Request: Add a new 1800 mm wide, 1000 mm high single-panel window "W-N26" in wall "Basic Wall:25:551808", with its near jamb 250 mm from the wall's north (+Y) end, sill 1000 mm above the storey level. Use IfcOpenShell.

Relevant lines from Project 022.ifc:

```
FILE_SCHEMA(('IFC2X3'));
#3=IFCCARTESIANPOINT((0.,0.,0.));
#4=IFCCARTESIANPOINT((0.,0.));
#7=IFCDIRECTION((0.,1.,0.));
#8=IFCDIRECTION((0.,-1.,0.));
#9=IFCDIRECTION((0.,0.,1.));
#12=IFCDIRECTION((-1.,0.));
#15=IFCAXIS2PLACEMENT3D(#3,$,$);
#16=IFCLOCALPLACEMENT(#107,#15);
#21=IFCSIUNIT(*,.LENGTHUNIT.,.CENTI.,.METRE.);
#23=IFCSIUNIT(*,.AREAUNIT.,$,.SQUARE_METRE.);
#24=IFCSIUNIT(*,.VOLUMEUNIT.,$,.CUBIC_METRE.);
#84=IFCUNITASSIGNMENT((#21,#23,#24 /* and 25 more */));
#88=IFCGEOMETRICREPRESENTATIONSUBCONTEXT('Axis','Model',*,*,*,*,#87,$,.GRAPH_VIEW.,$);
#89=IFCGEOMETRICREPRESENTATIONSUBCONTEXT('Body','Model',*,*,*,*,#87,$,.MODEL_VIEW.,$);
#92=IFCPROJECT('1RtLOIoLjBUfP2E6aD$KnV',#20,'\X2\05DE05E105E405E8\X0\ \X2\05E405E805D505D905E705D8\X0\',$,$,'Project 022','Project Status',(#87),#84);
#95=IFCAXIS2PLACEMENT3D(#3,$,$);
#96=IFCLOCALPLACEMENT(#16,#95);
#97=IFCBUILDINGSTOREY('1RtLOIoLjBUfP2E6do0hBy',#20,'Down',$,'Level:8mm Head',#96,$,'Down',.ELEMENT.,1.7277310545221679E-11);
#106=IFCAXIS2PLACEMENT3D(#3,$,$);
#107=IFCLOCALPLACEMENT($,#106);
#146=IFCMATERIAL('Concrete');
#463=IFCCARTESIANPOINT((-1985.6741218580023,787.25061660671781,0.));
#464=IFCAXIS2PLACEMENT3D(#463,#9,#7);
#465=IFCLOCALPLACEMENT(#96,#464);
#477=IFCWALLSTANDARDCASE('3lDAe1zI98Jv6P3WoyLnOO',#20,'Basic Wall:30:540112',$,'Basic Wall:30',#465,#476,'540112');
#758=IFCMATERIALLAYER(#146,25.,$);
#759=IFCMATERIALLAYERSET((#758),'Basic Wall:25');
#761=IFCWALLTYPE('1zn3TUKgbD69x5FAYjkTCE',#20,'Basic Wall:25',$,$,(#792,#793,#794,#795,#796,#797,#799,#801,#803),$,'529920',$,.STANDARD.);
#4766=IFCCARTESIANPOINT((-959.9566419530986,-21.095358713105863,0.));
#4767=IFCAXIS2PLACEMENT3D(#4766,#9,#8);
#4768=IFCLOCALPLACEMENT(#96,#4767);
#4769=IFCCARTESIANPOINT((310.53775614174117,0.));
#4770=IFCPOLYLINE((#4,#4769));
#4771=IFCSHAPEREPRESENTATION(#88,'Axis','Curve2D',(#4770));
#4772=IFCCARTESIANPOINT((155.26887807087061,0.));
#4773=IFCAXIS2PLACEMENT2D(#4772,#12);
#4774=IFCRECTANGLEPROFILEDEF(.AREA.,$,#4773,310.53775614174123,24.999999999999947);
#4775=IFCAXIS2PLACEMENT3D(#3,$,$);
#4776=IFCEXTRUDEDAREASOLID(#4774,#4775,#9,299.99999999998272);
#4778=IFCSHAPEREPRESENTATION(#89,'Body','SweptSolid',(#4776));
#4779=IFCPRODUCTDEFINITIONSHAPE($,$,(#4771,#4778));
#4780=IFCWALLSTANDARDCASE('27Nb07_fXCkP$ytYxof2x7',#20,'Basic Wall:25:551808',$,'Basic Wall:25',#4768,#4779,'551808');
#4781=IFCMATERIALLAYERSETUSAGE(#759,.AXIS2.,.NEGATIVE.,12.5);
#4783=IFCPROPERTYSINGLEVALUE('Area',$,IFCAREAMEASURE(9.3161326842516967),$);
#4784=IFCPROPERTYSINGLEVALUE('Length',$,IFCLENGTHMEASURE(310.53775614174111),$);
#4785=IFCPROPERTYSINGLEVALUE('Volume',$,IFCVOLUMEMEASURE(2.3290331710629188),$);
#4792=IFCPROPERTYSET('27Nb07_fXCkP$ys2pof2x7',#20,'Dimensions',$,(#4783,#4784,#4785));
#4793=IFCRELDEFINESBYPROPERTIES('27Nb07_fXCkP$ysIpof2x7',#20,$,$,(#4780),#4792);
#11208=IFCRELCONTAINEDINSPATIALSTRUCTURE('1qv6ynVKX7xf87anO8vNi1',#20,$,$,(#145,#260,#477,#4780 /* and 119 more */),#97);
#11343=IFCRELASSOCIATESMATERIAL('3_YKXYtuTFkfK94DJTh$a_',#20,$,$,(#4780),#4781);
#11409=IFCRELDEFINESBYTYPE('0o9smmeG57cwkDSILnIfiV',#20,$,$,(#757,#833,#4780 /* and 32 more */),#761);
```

```python
import numpy as np
import ifcopenshell
import ifcopenshell.api.feature
import ifcopenshell.api.geometry
import ifcopenshell.api.pset
import ifcopenshell.api.root
import ifcopenshell.api.spatial
import ifcopenshell.api.type
import ifcopenshell.geom
import ifcopenshell.util.element
import ifcopenshell.util.placement
import ifcopenshell.util.representation
import ifcopenshell.util.shape
import ifcopenshell.util.unit

model = ifcopenshell.open("Project 022.ifc")
unit_scale = ifcopenshell.util.unit.calculate_unit_scale(model)
area_scale = ifcopenshell.util.unit.calculate_unit_scale(model, "AREAUNIT")
volume_scale = ifcopenshell.util.unit.calculate_unit_scale(model, "VOLUMEUNIT")
settings = ifcopenshell.geom.settings()


def volume(element):
    """Net volume in cubic metres, openings subtracted."""
    shape = ifcopenshell.geom.create_shape(settings, element)
    return ifcopenshell.util.shape.get_volume(shape.geometry)


wall = model.by_guid("27Nb07_fXCkP$ytYxof2x7")
storey = ifcopenshell.util.element.get_container(wall, ifc_class="IfcBuildingStorey")
context = ifcopenshell.util.representation.get_context(model, "Model", "Body", "MODEL_VIEW")
before = volume(wall)

width, height, from_end, sill = 1.8, 1, 0.25, 1  # metres

# The wall runs along its own X axis, and the end named is its -X end.
wall_shape = ifcopenshell.geom.create_shape(settings, wall)
x, y, z = ifcopenshell.util.shape.get_vertices(wall_shape.geometry).T
start = x.min() + from_end
face, thickness = float(y.min()), float(y.max() - y.min())
wall_matrix = ifcopenshell.util.placement.get_local_placement(wall.ObjectPlacement)
level = ifcopenshell.util.placement.get_local_placement(storey.ObjectPlacement)[2, 3]


def in_wall(x, y):
    """Placement at x, y metres in the wall's axes, at sill height."""
    matrix = wall_matrix.copy()
    matrix[:, 3] = wall_matrix @ np.array([x / unit_scale, y / unit_scale, 0.0, 1.0])
    matrix[2, 3] = level + sill / unit_scale
    return matrix


# Opening: a box that overshoots both wall faces by 50 mm.
opening = ifcopenshell.api.root.create_entity(model, ifc_class="IfcOpeningElement")
box = ifcopenshell.api.geometry.add_wall_representation(
    model, context=context, length=width, height=height, thickness=thickness + 0.1
)
ifcopenshell.api.geometry.assign_representation(model, product=opening, representation=box)
ifcopenshell.api.geometry.edit_object_placement(model, product=opening, matrix=in_wall(start, face - 0.05), is_si=False)
ifcopenshell.api.feature.add_feature(model, feature=opening, element=wall)

window = ifcopenshell.api.root.create_entity(model, ifc_class="IfcWindow", name="W-N26")
window.OverallWidth, window.OverallHeight = width / unit_scale, height / unit_scale
body = ifcopenshell.api.geometry.add_window_representation(
    model,
    context=context,
    overall_width=window.OverallWidth,
    overall_height=window.OverallHeight,
    partition_type="SINGLE_PANEL",
)
ifcopenshell.api.geometry.assign_representation(model, product=window, representation=body)
ifcopenshell.api.spatial.assign_container(model, products=[window], relating_structure=storey)
fills = ifcopenshell.api.feature.add_filling(model, opening=opening, element=window)
fills.OwnerHistory = window.OwnerHistory  # required in IFC2X3

# IFC2X3 keeps the operation on the window style.
style = ifcopenshell.api.root.create_entity(model, ifc_class="IfcWindowStyle", name="W-N26")
style.OperationType, style.ConstructionType = "SINGLE_PANEL", "NOTDEFINED"
style.ParameterTakesPrecedence = style.Sizeable = False
ifcopenshell.api.type.assign_type(model, related_objects=[window], relating_type=style)

# Centre the window in the wall's thickness.
ifcopenshell.api.geometry.edit_object_placement(model, product=window, matrix=in_wall(start, face), is_si=False)
window_shape = ifcopenshell.geom.create_shape(settings, window)
depth = ifcopenshell.util.shape.get_vertices(window_shape.geometry)[:, 1]
offset = face + thickness / 2 - (depth.min() + depth.max()) / 2
ifcopenshell.api.geometry.edit_object_placement(model, product=window, matrix=in_wall(start, offset), is_si=False)

after = volume(wall)

# Update the wall's stored quantities.
pset = model.by_id(ifcopenshell.util.element.get_pset(wall, "Dimensions", should_inherit=False)["id"])
ifcopenshell.api.pset.edit_pset(model, pset=pset, properties={
    "Area": model.create_entity("IfcAreaMeasure", after / thickness / area_scale),
    "Volume": model.create_entity("IfcVolumeMeasure", after / volume_scale),
})

print(f"wall volume {before:.3f} -> {after:.3f} m3")

model.write("Project 022_edited.ifc")
```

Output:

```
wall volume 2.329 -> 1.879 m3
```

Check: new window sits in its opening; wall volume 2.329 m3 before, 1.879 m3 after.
